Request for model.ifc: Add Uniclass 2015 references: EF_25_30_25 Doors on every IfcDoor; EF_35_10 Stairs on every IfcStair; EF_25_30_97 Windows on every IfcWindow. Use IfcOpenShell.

First a look at what the model holds.

```python
import ifcopenshell

model = ifcopenshell.open("model.ifc")
print(model.schema)
print("classifications:", [c.Name for c in model.by_type("IfcClassification")])
for ifc_class in ("IfcDoor", "IfcRoof", "IfcStair", "IfcWall", "IfcWindow"):
    print(ifc_class, len(model.by_type(ifc_class)))
```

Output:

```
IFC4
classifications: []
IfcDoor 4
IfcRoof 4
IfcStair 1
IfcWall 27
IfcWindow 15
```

```python
import ifcopenshell
import ifcopenshell.api.classification

model = ifcopenshell.open("model.ifc")

system = ifcopenshell.api.classification.add_classification(model, classification="Uniclass 2015")

codes = {
    "IfcDoor": ("EF_25_30_25", "Doors"),
    "IfcStair": ("EF_35_10", "Stairs"),
    "IfcWindow": ("EF_25_30_97", "Windows"),
}
for ifc_class, (code, name) in codes.items():
    products = model.by_type(ifc_class)
    ifcopenshell.api.classification.add_reference(
        model, products=products, classification=system, identification=code, name=name
    )
    print(code, len(products))

model.write("model_v2.ifc")
```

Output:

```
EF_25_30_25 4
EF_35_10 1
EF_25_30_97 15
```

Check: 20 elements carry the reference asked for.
